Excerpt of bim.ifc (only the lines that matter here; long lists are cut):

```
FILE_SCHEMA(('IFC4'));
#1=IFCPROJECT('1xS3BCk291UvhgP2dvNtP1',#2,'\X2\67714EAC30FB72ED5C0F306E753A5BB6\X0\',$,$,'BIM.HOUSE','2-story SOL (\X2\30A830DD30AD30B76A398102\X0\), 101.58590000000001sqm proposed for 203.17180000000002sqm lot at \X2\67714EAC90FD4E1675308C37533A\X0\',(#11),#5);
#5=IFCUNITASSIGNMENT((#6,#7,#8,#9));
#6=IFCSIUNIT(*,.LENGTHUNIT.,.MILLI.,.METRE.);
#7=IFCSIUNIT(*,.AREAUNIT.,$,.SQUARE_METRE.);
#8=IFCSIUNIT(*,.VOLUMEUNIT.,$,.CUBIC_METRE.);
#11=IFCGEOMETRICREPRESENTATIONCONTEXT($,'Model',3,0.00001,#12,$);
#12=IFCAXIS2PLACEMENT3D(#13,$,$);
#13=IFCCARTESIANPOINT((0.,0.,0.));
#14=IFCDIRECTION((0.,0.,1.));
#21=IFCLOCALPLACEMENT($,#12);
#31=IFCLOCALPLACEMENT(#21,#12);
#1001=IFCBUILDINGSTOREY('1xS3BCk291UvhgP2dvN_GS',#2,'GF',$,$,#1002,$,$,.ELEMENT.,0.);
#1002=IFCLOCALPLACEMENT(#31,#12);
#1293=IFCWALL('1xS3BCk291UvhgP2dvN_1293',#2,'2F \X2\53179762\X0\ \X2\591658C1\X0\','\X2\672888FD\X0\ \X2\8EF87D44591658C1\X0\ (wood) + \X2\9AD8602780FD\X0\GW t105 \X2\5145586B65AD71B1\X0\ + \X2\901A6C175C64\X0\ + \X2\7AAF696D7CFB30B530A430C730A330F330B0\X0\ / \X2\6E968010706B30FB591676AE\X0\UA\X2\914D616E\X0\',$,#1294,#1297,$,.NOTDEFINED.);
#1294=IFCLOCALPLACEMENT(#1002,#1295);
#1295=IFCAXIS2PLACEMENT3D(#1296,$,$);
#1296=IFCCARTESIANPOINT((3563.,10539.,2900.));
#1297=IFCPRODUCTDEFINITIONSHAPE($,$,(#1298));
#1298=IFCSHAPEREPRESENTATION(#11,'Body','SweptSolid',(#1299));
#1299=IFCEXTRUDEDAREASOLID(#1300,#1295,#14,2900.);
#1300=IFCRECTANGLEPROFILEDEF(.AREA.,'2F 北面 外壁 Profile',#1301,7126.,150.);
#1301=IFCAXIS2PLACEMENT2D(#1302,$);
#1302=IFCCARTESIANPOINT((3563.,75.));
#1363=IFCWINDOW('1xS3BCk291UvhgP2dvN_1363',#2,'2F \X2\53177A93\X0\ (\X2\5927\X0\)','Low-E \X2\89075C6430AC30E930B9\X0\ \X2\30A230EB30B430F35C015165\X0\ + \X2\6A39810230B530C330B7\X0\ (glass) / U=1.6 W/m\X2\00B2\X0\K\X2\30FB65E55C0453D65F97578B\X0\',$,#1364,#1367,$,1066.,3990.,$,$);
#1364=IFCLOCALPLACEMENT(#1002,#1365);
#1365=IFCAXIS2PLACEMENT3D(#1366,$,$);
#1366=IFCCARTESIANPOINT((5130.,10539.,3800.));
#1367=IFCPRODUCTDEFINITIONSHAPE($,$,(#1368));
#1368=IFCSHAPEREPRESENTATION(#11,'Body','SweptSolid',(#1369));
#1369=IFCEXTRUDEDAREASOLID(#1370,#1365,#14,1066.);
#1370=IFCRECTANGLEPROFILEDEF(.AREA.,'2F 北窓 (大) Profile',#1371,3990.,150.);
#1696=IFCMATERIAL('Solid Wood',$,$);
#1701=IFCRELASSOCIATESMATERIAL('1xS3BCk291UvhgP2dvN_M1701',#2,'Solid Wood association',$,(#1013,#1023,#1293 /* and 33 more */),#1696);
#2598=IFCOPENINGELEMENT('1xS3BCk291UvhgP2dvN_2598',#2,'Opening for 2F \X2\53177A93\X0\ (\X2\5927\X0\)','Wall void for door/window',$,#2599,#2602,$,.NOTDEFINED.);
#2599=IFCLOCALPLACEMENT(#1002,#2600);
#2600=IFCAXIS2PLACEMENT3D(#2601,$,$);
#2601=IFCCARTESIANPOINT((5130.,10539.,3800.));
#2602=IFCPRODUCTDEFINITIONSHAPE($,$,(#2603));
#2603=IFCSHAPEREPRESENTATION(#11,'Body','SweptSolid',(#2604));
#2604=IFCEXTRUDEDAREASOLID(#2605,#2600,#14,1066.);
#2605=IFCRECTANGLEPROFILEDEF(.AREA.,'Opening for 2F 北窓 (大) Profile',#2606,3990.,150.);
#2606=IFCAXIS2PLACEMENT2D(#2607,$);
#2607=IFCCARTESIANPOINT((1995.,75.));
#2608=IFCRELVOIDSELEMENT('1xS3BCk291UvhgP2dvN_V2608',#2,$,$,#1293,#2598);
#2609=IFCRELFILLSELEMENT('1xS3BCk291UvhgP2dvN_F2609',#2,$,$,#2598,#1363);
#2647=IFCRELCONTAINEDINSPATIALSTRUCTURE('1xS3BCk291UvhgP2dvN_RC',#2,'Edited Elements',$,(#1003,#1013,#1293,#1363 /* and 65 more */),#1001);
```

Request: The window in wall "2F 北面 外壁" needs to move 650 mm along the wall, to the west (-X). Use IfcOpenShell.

```python
import ifcopenshell
import ifcopenshell.api.geometry
import ifcopenshell.util.placement

model = ifcopenshell.open("bim.ifc")

window = model.by_guid("1xS3BCk291UvhgP2dvN_1363")
opening = window.FillsVoids[0].RelatingOpeningElement
wall = opening.VoidsElements[0].RelatingBuildingElement

wall_matrix = ifcopenshell.util.placement.get_local_placement(wall.ObjectPlacement)
shift = wall_matrix[:3, 0] * -650.0
before = ifcopenshell.util.placement.get_local_placement(window.ObjectPlacement)[:3, 3].copy()

# The window is not placed relative to its opening, so move both.
for product in (opening, window):
    matrix = ifcopenshell.util.placement.get_local_placement(product.ObjectPlacement)
    matrix[:3, 3] += shift
    ifcopenshell.api.geometry.edit_object_placement(model, product=product, matrix=matrix, is_si=False)

after = ifcopenshell.util.placement.get_local_placement(window.ObjectPlacement)[:3, 3]
print("window moved by", (after - before).round(3) + 0.0)

model.write("bim_rev.ifc")
```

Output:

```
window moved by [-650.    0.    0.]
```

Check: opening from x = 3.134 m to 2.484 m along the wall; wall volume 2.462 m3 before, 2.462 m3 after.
